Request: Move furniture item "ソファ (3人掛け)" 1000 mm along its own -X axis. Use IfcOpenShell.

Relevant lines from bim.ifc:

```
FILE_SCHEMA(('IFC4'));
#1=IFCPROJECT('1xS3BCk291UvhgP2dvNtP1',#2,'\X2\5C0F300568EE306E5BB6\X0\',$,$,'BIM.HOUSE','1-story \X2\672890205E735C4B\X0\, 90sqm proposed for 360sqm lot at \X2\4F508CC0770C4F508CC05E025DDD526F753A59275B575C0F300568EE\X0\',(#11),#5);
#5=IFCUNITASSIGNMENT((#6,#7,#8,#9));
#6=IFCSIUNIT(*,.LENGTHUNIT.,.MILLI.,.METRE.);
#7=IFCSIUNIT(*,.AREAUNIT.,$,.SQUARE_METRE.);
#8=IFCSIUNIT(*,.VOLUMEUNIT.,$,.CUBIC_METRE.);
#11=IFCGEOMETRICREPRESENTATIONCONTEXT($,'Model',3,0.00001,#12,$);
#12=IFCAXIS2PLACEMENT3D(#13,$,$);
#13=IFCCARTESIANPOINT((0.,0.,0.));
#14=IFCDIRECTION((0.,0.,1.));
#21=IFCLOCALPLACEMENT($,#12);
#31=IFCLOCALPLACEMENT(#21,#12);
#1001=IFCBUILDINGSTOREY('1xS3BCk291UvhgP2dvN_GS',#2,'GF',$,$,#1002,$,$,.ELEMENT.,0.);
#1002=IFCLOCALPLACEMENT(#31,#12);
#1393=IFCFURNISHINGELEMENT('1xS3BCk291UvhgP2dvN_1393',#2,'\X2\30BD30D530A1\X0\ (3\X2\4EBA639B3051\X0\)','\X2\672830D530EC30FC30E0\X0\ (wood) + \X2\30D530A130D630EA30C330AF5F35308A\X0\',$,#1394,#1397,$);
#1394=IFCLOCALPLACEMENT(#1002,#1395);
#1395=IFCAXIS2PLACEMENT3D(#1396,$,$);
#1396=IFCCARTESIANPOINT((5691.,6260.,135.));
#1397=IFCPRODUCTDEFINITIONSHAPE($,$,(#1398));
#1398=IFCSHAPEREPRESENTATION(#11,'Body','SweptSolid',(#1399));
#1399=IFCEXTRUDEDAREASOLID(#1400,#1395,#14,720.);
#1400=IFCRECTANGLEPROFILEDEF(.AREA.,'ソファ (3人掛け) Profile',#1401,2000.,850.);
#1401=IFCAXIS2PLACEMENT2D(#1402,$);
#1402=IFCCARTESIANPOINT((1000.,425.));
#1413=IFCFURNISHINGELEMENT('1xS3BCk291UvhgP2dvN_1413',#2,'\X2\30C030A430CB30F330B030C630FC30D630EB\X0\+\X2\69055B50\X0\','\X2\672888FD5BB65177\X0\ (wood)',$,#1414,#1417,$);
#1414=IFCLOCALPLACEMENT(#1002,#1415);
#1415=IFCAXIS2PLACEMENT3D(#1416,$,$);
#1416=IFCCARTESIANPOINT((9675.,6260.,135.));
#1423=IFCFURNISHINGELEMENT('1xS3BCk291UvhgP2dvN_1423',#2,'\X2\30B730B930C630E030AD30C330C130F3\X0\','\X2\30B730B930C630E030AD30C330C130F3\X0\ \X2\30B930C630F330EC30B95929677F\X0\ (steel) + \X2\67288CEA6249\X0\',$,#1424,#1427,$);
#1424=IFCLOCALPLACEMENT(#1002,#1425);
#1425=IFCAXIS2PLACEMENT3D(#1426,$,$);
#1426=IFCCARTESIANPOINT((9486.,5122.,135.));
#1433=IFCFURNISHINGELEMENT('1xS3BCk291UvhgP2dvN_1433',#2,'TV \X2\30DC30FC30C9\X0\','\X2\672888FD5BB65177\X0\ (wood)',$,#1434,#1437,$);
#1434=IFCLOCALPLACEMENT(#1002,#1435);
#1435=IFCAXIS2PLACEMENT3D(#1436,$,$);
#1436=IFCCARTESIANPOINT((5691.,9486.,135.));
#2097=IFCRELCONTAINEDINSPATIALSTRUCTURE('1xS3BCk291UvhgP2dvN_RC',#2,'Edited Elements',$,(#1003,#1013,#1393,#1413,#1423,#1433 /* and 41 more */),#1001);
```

```python
import ifcopenshell
import ifcopenshell.api.geometry
import ifcopenshell.util.placement
import ifcopenshell.util.unit

model = ifcopenshell.open("bim.ifc")
unit_scale = ifcopenshell.util.unit.calculate_unit_scale(model)

item = model.by_guid("1xS3BCk291UvhgP2dvN_1393")
matrix = ifcopenshell.util.placement.get_local_placement(item.ObjectPlacement)
matrix[:3, 3] -= matrix[:3, 0] * 1 / unit_scale
ifcopenshell.api.geometry.edit_object_placement(model, product=item, matrix=matrix, is_si=False)

print(ifcopenshell.util.placement.get_local_placement(item.ObjectPlacement).round(3) + 0.0)

model.write("bim_v2.ifc")
```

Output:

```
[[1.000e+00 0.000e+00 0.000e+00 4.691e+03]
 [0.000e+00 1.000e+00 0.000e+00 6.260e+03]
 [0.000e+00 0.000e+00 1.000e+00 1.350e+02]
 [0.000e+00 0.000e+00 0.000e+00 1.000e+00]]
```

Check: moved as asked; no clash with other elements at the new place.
